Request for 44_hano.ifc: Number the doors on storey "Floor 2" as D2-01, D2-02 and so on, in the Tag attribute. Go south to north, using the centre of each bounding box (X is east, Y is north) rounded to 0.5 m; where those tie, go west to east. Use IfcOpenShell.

First a look at what the model holds.

```python
import ifcopenshell
import ifcopenshell.util.element
import ifcopenshell.util.placement

model = ifcopenshell.open("44_hano.ifc")
print(model.schema)
storey = next(s for s in model.by_type("IfcBuildingStorey") if s.Name == "Floor 2")
doors = [e for e in ifcopenshell.util.element.get_decomposition(storey) if e.is_a("IfcDoor")]
for e in sorted(doors, key=lambda e: e.id()):
    origin = ifcopenshell.util.placement.get_local_placement(e.ObjectPlacement)[:3, 3]
    print(e.id(), e.Tag, e.Name, origin.round(2) + 0.0, sep=" | ")
```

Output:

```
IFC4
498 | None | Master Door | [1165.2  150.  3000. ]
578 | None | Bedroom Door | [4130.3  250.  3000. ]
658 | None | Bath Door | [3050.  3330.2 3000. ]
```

```python
import ifcopenshell
import ifcopenshell.geom
import ifcopenshell.util.element
import ifcopenshell.util.shape

model = ifcopenshell.open("44_hano.ifc")
settings = ifcopenshell.geom.settings()
settings.set("use-world-coords", True)


def centre(element):
    shape = ifcopenshell.geom.create_shape(settings, element)
    return ifcopenshell.util.shape.get_bbox_centroid(shape.geometry)


storey = next(s for s in model.by_type("IfcBuildingStorey") if s.Name == "Floor 2")
doors = [e for e in ifcopenshell.util.element.get_decomposition(storey) if e.is_a("IfcDoor")]

# Insertion points can sit at a corner or the storey origin, so sort by the geometry (in metres).
centres = {e: centre(e) for e in doors}
doors.sort(key=lambda e: (round(centres[e][1] / 0.5), centres[e][0]))

for i, e in enumerate(doors, start=1):
    number = f"D2-{i:02d}"
    e.Tag = number
    print(e.id(), number)

model.write("44_hano_edited.ifc")
```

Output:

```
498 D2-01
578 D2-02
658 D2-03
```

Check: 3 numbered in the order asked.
